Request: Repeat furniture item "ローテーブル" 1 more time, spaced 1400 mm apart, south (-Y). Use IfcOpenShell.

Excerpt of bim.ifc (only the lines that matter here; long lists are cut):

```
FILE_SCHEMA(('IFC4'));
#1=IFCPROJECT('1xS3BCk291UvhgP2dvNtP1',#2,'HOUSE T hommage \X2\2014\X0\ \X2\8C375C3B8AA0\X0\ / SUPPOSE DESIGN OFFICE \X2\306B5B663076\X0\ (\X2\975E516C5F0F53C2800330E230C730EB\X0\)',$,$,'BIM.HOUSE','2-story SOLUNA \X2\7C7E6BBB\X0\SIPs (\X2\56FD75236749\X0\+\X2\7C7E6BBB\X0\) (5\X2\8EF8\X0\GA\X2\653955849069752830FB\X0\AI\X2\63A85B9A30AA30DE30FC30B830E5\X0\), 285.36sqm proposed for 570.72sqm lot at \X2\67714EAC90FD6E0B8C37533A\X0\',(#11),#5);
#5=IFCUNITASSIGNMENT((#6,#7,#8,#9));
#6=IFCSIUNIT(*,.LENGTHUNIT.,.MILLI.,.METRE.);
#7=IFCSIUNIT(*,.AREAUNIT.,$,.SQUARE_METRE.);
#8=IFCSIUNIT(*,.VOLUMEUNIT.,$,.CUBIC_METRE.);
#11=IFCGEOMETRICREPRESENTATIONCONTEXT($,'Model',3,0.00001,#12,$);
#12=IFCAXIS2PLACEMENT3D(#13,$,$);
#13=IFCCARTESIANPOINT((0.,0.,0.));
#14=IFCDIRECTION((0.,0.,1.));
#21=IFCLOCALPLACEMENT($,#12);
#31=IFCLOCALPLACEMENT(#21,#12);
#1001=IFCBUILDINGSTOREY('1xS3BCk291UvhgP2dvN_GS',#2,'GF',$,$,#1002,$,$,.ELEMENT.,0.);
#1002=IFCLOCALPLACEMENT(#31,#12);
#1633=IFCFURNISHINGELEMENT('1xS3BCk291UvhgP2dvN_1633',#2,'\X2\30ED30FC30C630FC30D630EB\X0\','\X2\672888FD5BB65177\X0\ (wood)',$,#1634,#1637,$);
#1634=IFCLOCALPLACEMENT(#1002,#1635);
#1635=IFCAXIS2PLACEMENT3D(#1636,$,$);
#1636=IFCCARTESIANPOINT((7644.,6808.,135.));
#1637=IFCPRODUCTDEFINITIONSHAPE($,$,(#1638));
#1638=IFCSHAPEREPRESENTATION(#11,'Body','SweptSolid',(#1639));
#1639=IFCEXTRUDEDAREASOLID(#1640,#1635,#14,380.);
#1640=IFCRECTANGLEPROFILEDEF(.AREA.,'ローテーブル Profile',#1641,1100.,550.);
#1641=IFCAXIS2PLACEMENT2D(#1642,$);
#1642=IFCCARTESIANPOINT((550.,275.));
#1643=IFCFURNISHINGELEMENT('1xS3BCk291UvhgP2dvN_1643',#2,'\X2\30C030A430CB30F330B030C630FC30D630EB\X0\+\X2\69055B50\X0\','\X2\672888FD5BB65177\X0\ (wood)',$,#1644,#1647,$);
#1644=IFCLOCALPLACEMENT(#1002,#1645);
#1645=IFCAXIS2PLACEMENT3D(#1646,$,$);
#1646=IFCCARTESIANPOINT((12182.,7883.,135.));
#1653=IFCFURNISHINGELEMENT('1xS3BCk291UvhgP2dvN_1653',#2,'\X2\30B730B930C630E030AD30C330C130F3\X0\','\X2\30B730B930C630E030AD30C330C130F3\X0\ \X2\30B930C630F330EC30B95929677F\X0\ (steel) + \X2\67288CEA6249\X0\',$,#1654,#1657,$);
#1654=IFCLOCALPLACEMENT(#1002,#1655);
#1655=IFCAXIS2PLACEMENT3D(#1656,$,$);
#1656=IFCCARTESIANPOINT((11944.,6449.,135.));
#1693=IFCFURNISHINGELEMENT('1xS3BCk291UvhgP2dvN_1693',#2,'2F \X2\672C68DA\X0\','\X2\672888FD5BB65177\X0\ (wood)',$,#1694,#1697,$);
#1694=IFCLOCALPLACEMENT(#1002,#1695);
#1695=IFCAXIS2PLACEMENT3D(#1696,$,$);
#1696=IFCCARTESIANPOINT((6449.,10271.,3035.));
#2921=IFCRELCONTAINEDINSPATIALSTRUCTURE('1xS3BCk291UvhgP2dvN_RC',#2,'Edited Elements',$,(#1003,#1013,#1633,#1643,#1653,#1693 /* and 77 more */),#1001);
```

```python
import numpy as np
import ifcopenshell
import ifcopenshell.api.geometry
import ifcopenshell.api.root
import ifcopenshell.util.element
import ifcopenshell.util.placement

model = ifcopenshell.open("bim.ifc")


def reuse_history(source, copy):
    """copy_class also copies each property set's owner history, people and application; keep the originals."""
    for rel in copy.IsDefinedBy:
        if rel.is_a("IfcRelDefinesByProperties") and (history := rel.RelatingPropertyDefinition.OwnerHistory):
            rel.RelatingPropertyDefinition.OwnerHistory = source.OwnerHistory
            ifcopenshell.util.element.remove_deep2(model, history)


source = model.by_guid("1xS3BCk291UvhgP2dvN_1633")
base = ifcopenshell.util.placement.get_local_placement(source.ObjectPlacement)
step = np.array([0.0, -1.0, 0.0]) * 1400.0

for i in range(1, 2):
    copy = ifcopenshell.api.root.copy_class(model, product=source)
    copy.Representation = ifcopenshell.util.element.copy_deep(
        model, source.Representation, exclude=["IfcGeometricRepresentationContext", "IfcRepresentationMap"]
    )
    reuse_history(source, copy)
    matrix = base.copy()
    matrix[:3, 3] += i * step
    print("added at", matrix[:3, 3].round(3) + 0.0)
    ifcopenshell.api.geometry.edit_object_placement(model, product=copy, matrix=matrix, is_si=False)

model.write("bim-out.ifc")
```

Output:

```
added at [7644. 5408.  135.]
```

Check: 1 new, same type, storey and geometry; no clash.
